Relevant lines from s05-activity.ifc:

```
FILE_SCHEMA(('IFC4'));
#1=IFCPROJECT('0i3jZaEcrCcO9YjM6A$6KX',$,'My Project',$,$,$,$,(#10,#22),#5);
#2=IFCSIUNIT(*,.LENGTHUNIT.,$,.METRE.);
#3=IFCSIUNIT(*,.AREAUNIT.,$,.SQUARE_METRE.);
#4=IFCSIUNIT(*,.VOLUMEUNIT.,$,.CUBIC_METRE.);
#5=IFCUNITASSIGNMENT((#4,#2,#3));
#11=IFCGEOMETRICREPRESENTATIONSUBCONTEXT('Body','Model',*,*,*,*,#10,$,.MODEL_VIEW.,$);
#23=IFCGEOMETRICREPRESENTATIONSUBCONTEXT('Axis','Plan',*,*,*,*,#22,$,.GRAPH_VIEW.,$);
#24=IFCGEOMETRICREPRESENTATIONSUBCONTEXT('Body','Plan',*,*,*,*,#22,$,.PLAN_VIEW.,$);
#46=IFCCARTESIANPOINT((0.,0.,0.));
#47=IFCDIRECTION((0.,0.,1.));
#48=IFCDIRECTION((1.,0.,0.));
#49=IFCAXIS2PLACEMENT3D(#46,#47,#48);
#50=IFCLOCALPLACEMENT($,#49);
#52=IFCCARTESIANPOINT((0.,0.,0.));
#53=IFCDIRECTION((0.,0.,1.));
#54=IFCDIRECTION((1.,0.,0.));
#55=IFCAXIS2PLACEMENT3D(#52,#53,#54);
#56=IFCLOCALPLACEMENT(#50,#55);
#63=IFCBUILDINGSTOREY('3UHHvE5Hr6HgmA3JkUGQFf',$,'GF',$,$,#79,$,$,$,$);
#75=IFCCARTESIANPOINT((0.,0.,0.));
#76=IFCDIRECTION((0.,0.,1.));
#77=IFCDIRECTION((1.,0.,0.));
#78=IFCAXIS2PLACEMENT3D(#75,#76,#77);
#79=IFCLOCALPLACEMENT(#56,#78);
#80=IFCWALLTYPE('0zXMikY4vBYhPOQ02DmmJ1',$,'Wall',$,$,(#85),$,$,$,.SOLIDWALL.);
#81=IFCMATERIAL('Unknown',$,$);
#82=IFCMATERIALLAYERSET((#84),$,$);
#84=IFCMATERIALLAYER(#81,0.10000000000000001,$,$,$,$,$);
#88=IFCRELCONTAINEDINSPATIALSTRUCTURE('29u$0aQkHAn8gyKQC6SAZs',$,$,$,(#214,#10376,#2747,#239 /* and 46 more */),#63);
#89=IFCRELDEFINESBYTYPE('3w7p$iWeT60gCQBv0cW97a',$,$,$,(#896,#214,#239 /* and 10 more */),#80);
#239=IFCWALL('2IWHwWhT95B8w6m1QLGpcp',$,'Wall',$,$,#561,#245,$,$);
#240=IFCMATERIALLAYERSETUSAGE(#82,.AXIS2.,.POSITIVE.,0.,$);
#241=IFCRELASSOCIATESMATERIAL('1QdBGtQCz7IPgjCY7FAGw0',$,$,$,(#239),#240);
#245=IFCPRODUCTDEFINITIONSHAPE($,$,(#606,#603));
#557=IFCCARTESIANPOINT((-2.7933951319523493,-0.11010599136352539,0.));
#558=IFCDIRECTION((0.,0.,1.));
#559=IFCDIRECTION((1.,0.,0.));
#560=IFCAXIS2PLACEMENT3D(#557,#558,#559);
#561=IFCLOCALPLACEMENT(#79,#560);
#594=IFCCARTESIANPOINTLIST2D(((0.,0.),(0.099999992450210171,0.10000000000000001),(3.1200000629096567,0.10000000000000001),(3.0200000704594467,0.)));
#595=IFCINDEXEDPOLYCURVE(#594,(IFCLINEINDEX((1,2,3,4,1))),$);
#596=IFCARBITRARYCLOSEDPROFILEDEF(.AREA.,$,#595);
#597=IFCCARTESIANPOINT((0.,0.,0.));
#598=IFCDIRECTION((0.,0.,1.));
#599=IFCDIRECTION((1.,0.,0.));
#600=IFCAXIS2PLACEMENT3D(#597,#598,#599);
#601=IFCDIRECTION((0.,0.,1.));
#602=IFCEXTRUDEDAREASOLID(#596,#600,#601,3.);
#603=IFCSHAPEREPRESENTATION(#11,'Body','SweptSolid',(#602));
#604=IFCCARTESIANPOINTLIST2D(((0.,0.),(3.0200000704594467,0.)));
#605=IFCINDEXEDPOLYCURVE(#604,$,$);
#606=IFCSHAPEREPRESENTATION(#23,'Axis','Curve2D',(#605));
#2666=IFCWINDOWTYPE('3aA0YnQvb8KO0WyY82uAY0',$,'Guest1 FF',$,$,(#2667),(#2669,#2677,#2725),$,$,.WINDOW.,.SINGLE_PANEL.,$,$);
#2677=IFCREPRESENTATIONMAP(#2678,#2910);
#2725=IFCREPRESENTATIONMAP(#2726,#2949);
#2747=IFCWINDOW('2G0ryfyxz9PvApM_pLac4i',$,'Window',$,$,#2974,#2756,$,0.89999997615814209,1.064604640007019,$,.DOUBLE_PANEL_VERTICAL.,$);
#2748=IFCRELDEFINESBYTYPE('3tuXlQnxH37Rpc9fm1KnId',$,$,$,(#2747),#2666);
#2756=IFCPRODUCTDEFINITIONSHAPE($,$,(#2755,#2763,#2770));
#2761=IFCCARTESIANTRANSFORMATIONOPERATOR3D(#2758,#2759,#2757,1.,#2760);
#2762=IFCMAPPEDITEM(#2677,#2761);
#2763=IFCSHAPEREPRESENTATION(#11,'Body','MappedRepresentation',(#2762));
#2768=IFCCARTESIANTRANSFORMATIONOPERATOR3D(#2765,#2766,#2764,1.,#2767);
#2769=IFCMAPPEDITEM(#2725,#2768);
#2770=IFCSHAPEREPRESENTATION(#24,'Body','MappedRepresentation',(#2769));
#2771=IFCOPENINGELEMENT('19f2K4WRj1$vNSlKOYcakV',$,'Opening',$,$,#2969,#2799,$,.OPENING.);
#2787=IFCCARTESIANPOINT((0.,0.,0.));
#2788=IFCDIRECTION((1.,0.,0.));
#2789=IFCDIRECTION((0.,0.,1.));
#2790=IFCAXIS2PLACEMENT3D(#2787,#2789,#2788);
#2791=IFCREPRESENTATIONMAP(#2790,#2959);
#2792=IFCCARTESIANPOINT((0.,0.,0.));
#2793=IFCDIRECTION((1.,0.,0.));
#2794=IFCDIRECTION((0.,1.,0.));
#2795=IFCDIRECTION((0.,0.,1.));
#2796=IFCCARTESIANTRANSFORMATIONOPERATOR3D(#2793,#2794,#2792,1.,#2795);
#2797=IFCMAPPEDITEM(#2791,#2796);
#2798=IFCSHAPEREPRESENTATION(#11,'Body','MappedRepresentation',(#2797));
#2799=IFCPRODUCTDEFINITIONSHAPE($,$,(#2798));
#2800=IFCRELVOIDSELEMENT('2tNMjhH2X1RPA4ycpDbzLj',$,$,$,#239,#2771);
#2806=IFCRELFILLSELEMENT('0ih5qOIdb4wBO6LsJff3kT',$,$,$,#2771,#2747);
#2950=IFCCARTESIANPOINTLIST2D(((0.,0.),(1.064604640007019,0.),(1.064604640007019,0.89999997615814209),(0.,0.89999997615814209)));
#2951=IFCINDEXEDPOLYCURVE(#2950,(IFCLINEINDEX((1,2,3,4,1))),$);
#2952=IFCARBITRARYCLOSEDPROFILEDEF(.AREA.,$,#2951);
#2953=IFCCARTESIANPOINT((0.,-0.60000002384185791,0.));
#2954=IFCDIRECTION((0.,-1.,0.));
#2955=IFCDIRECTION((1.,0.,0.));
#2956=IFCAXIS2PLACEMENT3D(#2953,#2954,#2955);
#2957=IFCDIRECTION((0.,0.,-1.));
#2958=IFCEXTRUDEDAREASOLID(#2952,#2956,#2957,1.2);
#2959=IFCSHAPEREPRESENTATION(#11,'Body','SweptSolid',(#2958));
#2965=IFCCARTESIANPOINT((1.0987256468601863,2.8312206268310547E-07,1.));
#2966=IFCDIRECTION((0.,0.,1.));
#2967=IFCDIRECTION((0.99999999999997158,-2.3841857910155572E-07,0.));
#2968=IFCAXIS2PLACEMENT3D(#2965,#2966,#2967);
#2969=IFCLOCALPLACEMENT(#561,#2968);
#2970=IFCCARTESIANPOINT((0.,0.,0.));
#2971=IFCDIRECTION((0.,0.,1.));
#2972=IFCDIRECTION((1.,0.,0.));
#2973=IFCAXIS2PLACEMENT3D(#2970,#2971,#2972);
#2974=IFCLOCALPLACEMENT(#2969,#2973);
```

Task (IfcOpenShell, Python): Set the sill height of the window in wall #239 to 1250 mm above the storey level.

```python
import numpy as np
import ifcopenshell
import ifcopenshell.api.geometry
import ifcopenshell.geom
import ifcopenshell.util.element
import ifcopenshell.util.placement
import ifcopenshell.util.shape
import ifcopenshell.util.unit

model = ifcopenshell.open("s05-activity.ifc")
unit_scale = ifcopenshell.util.unit.calculate_unit_scale(model)

window = model.by_guid("2G0ryfyxz9PvApM_pLac4i")
opening = window.FillsVoids[0].RelatingOpeningElement
storey = ifcopenshell.util.element.get_container(window, ifc_class="IfcBuildingStorey")
level = ifcopenshell.util.placement.get_local_placement(storey.ObjectPlacement)[2, 3]

# The opening's origin need not be at the sill, so measure its lowest point.
shape = ifcopenshell.geom.create_shape(ifcopenshell.geom.settings(), opening)
bottom = ifcopenshell.util.shape.get_shape_bottom_elevation(shape, shape.geometry) / unit_scale
dz = level + 1.25 - bottom

shift = np.array([0.0, 0.0, dz])
# The window is placed relative to its opening, so it follows when the opening moves.
matrix = ifcopenshell.util.placement.get_local_placement(opening.ObjectPlacement)
matrix[:3, 3] += shift
ifcopenshell.api.geometry.edit_object_placement(
    model, product=opening, matrix=matrix, is_si=False, should_transform_children=True
)

print(f"moved by {dz * unit_scale:+.3f} m")

model.write("s05-activity_updated.ifc")
```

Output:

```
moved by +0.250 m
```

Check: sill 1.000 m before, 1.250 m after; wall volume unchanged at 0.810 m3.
